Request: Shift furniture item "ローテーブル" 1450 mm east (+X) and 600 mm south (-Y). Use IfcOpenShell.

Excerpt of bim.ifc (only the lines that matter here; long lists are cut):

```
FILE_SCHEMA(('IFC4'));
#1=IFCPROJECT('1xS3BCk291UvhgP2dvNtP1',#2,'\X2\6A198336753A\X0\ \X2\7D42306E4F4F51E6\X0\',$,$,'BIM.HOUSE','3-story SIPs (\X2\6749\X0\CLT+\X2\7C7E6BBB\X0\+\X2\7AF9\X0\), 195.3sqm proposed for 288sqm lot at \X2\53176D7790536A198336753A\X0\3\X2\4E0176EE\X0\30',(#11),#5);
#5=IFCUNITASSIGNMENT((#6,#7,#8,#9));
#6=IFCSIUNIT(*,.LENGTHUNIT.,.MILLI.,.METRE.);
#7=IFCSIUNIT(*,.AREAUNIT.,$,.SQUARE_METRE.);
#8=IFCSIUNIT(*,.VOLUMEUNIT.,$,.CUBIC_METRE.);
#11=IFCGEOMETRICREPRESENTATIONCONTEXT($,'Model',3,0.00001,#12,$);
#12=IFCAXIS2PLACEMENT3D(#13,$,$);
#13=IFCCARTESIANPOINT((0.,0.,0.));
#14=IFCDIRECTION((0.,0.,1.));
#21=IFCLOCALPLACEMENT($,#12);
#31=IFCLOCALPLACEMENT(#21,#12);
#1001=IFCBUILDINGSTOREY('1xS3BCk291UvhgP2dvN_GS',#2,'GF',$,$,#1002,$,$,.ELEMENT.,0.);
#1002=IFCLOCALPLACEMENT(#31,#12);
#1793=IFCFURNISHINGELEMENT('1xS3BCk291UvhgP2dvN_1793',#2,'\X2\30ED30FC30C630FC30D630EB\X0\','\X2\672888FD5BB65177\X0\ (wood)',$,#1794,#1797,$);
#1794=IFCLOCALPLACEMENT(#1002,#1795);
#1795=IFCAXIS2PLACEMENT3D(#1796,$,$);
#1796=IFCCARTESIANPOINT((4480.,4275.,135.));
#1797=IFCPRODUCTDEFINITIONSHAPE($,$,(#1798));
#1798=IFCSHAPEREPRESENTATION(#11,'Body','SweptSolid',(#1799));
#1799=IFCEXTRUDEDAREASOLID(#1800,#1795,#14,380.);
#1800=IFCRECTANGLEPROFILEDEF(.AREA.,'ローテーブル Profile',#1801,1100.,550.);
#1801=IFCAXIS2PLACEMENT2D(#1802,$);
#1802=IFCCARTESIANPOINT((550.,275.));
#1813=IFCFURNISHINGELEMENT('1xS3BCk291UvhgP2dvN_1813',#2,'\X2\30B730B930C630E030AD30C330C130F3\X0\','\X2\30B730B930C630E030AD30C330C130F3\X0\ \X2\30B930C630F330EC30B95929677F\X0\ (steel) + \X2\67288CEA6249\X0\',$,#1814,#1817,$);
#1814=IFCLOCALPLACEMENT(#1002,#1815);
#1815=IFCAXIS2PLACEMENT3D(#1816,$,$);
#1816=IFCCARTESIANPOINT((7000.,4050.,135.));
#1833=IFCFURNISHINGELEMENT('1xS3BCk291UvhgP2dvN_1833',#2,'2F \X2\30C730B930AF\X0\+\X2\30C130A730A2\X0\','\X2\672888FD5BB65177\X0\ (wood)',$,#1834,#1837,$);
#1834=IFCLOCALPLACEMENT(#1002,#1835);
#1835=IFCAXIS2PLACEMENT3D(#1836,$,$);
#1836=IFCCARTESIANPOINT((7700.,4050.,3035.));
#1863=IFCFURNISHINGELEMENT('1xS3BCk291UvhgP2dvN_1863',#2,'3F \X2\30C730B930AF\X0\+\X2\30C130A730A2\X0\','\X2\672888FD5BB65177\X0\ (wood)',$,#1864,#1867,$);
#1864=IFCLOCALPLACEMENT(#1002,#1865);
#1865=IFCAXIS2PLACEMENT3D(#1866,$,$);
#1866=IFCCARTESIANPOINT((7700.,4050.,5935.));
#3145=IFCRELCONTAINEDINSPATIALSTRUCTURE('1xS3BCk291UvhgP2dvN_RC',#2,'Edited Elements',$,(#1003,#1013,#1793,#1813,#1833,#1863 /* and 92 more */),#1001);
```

```python
import ifcopenshell
import ifcopenshell.api.geometry
import ifcopenshell.util.placement
import ifcopenshell.util.unit

model = ifcopenshell.open("bim.ifc")
unit_scale = ifcopenshell.util.unit.calculate_unit_scale(model)

item = model.by_guid("1xS3BCk291UvhgP2dvN_1793")
matrix = ifcopenshell.util.placement.get_local_placement(item.ObjectPlacement)
matrix[0, 3] += 1.45 / unit_scale
matrix[1, 3] -= 0.6 / unit_scale
ifcopenshell.api.geometry.edit_object_placement(model, product=item, matrix=matrix, is_si=False)

print(ifcopenshell.util.placement.get_local_placement(item.ObjectPlacement).round(3) + 0.0)

model.write("bim_edited.ifc")
```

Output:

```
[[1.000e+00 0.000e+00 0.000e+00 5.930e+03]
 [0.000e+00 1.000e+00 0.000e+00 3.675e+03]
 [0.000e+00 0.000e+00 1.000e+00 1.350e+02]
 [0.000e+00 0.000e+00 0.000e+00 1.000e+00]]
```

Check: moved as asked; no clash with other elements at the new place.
